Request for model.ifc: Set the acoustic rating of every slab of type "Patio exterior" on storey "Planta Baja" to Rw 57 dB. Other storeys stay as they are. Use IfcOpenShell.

First a look at what the model holds.

```python
import ifcopenshell
import ifcopenshell.util.element

model = ifcopenshell.open("model.ifc")
print(model.schema)
storey = next(s for s in model.by_type("IfcBuildingStorey") if s.Name == "Planta Baja")
slabs = [e for e in ifcopenshell.util.element.get_decomposition(storey) if e.is_a("IfcSlab")]
seen = {}
for e in slabs:
    element_type = ifcopenshell.util.element.get_type(e)
    key = (element_type.Name if element_type != e and element_type else None, ifcopenshell.util.element.get_pset(e, "Pset_SlabCommon", "AcousticRating"))
    seen[key] = seen.get(key, 0) + 1
for (name, value), count in sorted(seen.items(), key=str):
    print(count, "x", name, "|", value)
```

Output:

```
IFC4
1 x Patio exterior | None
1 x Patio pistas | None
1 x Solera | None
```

```python
import ifcopenshell
import ifcopenshell.api.pset
import ifcopenshell.util.element

model = ifcopenshell.open("model.ifc")

storey = next(s for s in model.by_type("IfcBuildingStorey") if s.Name == "Planta Baja")
slabs = [e for e in ifcopenshell.util.element.get_decomposition(storey) if e.is_a("IfcSlab")]

count = 0
for e in slabs:
    element_type = ifcopenshell.util.element.get_type(e)
    if element_type in (None, e) or element_type.Name != "Patio exterior":
        continue
    # add_pset returns the element's existing set when there is one.
    pset = ifcopenshell.api.pset.add_pset(model, product=e, name="Pset_SlabCommon")
    ifcopenshell.api.pset.edit_pset(model, pset=pset, properties={"AcousticRating": "Rw 57 dB"})
    count += 1

print(count, "slabs updated")

model.write("model_v2.ifc")
```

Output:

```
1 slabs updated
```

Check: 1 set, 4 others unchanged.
